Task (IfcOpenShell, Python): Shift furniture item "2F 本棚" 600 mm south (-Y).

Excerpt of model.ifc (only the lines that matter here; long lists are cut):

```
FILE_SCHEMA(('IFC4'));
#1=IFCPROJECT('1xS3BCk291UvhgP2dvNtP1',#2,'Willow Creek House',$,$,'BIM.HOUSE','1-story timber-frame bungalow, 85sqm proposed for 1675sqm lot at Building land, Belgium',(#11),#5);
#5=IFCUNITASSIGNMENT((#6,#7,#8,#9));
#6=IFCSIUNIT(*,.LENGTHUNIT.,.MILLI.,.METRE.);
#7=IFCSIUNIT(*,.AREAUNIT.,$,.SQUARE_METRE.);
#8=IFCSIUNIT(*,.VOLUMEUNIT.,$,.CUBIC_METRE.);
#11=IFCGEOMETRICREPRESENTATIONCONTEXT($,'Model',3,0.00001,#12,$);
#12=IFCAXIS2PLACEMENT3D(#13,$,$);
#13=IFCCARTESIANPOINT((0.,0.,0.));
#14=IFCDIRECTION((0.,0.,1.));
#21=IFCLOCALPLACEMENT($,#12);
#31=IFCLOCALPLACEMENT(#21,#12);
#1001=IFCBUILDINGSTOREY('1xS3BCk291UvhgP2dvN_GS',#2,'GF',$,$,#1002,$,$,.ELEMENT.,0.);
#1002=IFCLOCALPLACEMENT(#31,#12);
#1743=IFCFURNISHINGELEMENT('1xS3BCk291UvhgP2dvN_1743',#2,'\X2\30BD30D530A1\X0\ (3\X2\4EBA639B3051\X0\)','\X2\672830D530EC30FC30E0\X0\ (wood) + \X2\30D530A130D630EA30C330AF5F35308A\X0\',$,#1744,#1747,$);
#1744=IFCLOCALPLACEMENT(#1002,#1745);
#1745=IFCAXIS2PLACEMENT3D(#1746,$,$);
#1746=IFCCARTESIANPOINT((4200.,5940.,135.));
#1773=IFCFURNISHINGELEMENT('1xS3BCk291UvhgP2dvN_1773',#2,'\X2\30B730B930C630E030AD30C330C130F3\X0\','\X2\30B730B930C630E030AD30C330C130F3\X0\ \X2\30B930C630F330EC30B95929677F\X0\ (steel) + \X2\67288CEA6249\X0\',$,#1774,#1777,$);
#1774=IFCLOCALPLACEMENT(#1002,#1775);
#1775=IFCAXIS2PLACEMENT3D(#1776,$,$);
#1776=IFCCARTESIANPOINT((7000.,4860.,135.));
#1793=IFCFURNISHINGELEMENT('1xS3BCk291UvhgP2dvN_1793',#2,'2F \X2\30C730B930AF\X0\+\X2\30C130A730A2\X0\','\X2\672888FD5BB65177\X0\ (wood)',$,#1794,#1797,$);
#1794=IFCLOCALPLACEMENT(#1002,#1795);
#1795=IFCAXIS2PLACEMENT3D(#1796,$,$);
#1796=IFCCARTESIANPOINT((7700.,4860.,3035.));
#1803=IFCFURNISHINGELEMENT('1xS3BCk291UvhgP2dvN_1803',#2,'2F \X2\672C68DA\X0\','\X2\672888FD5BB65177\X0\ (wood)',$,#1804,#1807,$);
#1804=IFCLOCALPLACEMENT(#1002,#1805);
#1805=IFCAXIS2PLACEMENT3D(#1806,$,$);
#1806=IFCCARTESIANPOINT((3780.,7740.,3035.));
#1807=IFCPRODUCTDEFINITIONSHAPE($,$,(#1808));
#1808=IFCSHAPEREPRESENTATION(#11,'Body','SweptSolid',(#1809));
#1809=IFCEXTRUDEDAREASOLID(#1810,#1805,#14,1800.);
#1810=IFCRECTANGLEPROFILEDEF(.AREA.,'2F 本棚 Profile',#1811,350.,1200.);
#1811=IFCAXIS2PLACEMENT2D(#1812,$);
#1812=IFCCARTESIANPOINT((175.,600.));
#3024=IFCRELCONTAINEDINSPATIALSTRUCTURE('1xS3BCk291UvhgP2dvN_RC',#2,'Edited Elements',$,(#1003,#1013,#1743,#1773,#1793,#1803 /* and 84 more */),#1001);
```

```python
import ifcopenshell
import ifcopenshell.api.geometry
import ifcopenshell.util.placement
import ifcopenshell.util.unit

model = ifcopenshell.open("model.ifc")
unit_scale = ifcopenshell.util.unit.calculate_unit_scale(model)

item = model.by_id(1803)
matrix = ifcopenshell.util.placement.get_local_placement(item.ObjectPlacement)
matrix[1, 3] -= 0.6 / unit_scale
ifcopenshell.api.geometry.edit_object_placement(model, product=item, matrix=matrix, is_si=False)

print(ifcopenshell.util.placement.get_local_placement(item.ObjectPlacement).round(3) + 0.0)

model.write("model_updated.ifc")
```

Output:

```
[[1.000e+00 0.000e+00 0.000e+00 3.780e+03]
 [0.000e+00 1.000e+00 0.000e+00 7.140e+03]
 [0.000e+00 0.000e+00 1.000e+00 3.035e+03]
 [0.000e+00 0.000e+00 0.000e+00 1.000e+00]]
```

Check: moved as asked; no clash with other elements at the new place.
